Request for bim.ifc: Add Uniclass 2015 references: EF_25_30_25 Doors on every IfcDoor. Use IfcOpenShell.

First a look at what the model holds.

```python
import ifcopenshell

model = ifcopenshell.open("bim.ifc")
print(model.schema)
print("classifications:", [c.Name for c in model.by_type("IfcClassification")])
for ifc_class in ("IfcDoor", "IfcRoof", "IfcStair", "IfcWall", "IfcWindow"):
    print(ifc_class, len(model.by_type(ifc_class)))
```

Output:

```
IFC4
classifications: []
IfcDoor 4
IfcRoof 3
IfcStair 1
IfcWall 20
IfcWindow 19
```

```python
import ifcopenshell
import ifcopenshell.api.classification

model = ifcopenshell.open("bim.ifc")

system = ifcopenshell.api.classification.add_classification(model, classification="Uniclass 2015")

codes = {
    "IfcDoor": ("EF_25_30_25", "Doors"),
}
for ifc_class, (code, name) in codes.items():
    products = model.by_type(ifc_class)
    ifcopenshell.api.classification.add_reference(
        model, products=products, classification=system, identification=code, name=name
    )
    print(code, len(products))

model.write("bim_rev.ifc")
```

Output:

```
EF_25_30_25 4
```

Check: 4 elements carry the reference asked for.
